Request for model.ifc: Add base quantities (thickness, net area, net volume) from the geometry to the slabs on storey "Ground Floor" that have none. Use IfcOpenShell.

First a look at what the model holds.

```python
import ifcopenshell
import ifcopenshell.util.element
import ifcopenshell.util.unit

model = ifcopenshell.open("model.ifc")
print(model.schema)
for unit_type in ("LENGTHUNIT", "AREAUNIT", "VOLUMEUNIT"):
    print(unit_type, ifcopenshell.util.unit.calculate_unit_scale(model, unit_type))
storey = next(s for s in model.by_type("IfcBuildingStorey") if s.Name == "Ground Floor")
slabs = [e for e in ifcopenshell.util.element.get_decomposition(storey) if e.is_a("IfcSlab")]
for e in sorted(slabs, key=lambda e: e.id()):
    print(e.id(), e.is_a(), e.Name, list(ifcopenshell.util.element.get_psets(e, qtos_only=True)), sep=" | ")
```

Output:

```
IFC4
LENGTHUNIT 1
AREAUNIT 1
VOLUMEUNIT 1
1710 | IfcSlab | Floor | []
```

```python
import ifcopenshell
import ifcopenshell.api.pset
import ifcopenshell.geom
import ifcopenshell.util.element
import ifcopenshell.util.shape
import ifcopenshell.util.unit

model = ifcopenshell.open("model.ifc")
unit_scale = ifcopenshell.util.unit.calculate_unit_scale(model)
area_scale = ifcopenshell.util.unit.calculate_unit_scale(model, "AREAUNIT")
volume_scale = ifcopenshell.util.unit.calculate_unit_scale(model, "VOLUMEUNIT")
settings = ifcopenshell.geom.settings()

storey = next(s for s in model.by_type("IfcBuildingStorey") if s.Name == "Ground Floor")
slabs = [e for e in ifcopenshell.util.element.get_decomposition(storey) if e.is_a("IfcSlab")]

for e in sorted(slabs, key=lambda e: e.id()):
    if ifcopenshell.util.element.get_psets(e, qtos_only=True, should_inherit=False):
        continue
    # Geometry comes back in metres, in the element's own axes.
    shape = ifcopenshell.geom.create_shape(settings, e)
    values = {
        "Width": ifcopenshell.util.shape.get_z(shape.geometry) / unit_scale,
        "NetArea": ifcopenshell.util.shape.get_footprint_area(shape.geometry) / area_scale,
        "NetVolume": ifcopenshell.util.shape.get_volume(shape.geometry) / volume_scale,
    }
    qto = ifcopenshell.api.pset.add_qto(model, product=e, name="Qto_SlabBaseQuantities")
    ifcopenshell.api.pset.edit_qto(model, qto=qto, properties=values)
    print(e.id(), {k: round(v, 3) for k, v in values.items()})

model.write("model-out.ifc")
```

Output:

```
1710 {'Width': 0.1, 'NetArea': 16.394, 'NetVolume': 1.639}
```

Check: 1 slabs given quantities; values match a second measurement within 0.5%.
